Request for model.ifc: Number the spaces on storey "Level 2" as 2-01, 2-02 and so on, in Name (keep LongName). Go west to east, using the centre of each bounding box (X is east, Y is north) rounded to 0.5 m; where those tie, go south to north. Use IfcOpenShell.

First a look at what the model holds.

```python
import ifcopenshell
import ifcopenshell.util.element
import ifcopenshell.util.placement

model = ifcopenshell.open("model.ifc")
print(model.schema)
storey = next(s for s in model.by_type("IfcBuildingStorey") if s.Name == "Level 2")
spaces = [e for e in ifcopenshell.util.element.get_decomposition(storey) if e.is_a("IfcSpace")]
for e in sorted(spaces, key=lambda e: e.id()):
    origin = ifcopenshell.util.placement.get_local_placement(e.ObjectPlacement)[:3, 3]
    print(e.id(), e.Name, e.LongName, origin.round(2) + 0.0, sep=" | ")
```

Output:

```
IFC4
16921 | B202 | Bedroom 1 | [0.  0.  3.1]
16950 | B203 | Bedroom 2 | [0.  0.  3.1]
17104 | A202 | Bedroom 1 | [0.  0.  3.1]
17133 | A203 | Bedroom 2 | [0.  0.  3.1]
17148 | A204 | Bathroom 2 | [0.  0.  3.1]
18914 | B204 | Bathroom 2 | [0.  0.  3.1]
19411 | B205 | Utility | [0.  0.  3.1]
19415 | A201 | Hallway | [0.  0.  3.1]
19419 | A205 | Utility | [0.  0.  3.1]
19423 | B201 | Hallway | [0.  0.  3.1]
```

```python
import ifcopenshell
import ifcopenshell.geom
import ifcopenshell.util.element
import ifcopenshell.util.shape

model = ifcopenshell.open("model.ifc")
settings = ifcopenshell.geom.settings()
settings.set("use-world-coords", True)


def centre(element):
    shape = ifcopenshell.geom.create_shape(settings, element)
    return ifcopenshell.util.shape.get_bbox_centroid(shape.geometry)


storey = next(s for s in model.by_type("IfcBuildingStorey") if s.Name == "Level 2")
spaces = [e for e in ifcopenshell.util.element.get_decomposition(storey) if e.is_a("IfcSpace")]

# Insertion points can sit at a corner or the storey origin, so sort by the geometry (in metres).
centres = {e: centre(e) for e in spaces}
spaces.sort(key=lambda e: (round(centres[e][0] / 0.5), centres[e][1]))

for i, e in enumerate(spaces, start=1):
    number = f"2-{i:02d}"
    e.Name = number
    print(e.id(), number)

model.write("model_rev.ifc")
```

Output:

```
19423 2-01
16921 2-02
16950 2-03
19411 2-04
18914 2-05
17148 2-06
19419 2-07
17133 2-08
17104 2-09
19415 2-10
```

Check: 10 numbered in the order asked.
